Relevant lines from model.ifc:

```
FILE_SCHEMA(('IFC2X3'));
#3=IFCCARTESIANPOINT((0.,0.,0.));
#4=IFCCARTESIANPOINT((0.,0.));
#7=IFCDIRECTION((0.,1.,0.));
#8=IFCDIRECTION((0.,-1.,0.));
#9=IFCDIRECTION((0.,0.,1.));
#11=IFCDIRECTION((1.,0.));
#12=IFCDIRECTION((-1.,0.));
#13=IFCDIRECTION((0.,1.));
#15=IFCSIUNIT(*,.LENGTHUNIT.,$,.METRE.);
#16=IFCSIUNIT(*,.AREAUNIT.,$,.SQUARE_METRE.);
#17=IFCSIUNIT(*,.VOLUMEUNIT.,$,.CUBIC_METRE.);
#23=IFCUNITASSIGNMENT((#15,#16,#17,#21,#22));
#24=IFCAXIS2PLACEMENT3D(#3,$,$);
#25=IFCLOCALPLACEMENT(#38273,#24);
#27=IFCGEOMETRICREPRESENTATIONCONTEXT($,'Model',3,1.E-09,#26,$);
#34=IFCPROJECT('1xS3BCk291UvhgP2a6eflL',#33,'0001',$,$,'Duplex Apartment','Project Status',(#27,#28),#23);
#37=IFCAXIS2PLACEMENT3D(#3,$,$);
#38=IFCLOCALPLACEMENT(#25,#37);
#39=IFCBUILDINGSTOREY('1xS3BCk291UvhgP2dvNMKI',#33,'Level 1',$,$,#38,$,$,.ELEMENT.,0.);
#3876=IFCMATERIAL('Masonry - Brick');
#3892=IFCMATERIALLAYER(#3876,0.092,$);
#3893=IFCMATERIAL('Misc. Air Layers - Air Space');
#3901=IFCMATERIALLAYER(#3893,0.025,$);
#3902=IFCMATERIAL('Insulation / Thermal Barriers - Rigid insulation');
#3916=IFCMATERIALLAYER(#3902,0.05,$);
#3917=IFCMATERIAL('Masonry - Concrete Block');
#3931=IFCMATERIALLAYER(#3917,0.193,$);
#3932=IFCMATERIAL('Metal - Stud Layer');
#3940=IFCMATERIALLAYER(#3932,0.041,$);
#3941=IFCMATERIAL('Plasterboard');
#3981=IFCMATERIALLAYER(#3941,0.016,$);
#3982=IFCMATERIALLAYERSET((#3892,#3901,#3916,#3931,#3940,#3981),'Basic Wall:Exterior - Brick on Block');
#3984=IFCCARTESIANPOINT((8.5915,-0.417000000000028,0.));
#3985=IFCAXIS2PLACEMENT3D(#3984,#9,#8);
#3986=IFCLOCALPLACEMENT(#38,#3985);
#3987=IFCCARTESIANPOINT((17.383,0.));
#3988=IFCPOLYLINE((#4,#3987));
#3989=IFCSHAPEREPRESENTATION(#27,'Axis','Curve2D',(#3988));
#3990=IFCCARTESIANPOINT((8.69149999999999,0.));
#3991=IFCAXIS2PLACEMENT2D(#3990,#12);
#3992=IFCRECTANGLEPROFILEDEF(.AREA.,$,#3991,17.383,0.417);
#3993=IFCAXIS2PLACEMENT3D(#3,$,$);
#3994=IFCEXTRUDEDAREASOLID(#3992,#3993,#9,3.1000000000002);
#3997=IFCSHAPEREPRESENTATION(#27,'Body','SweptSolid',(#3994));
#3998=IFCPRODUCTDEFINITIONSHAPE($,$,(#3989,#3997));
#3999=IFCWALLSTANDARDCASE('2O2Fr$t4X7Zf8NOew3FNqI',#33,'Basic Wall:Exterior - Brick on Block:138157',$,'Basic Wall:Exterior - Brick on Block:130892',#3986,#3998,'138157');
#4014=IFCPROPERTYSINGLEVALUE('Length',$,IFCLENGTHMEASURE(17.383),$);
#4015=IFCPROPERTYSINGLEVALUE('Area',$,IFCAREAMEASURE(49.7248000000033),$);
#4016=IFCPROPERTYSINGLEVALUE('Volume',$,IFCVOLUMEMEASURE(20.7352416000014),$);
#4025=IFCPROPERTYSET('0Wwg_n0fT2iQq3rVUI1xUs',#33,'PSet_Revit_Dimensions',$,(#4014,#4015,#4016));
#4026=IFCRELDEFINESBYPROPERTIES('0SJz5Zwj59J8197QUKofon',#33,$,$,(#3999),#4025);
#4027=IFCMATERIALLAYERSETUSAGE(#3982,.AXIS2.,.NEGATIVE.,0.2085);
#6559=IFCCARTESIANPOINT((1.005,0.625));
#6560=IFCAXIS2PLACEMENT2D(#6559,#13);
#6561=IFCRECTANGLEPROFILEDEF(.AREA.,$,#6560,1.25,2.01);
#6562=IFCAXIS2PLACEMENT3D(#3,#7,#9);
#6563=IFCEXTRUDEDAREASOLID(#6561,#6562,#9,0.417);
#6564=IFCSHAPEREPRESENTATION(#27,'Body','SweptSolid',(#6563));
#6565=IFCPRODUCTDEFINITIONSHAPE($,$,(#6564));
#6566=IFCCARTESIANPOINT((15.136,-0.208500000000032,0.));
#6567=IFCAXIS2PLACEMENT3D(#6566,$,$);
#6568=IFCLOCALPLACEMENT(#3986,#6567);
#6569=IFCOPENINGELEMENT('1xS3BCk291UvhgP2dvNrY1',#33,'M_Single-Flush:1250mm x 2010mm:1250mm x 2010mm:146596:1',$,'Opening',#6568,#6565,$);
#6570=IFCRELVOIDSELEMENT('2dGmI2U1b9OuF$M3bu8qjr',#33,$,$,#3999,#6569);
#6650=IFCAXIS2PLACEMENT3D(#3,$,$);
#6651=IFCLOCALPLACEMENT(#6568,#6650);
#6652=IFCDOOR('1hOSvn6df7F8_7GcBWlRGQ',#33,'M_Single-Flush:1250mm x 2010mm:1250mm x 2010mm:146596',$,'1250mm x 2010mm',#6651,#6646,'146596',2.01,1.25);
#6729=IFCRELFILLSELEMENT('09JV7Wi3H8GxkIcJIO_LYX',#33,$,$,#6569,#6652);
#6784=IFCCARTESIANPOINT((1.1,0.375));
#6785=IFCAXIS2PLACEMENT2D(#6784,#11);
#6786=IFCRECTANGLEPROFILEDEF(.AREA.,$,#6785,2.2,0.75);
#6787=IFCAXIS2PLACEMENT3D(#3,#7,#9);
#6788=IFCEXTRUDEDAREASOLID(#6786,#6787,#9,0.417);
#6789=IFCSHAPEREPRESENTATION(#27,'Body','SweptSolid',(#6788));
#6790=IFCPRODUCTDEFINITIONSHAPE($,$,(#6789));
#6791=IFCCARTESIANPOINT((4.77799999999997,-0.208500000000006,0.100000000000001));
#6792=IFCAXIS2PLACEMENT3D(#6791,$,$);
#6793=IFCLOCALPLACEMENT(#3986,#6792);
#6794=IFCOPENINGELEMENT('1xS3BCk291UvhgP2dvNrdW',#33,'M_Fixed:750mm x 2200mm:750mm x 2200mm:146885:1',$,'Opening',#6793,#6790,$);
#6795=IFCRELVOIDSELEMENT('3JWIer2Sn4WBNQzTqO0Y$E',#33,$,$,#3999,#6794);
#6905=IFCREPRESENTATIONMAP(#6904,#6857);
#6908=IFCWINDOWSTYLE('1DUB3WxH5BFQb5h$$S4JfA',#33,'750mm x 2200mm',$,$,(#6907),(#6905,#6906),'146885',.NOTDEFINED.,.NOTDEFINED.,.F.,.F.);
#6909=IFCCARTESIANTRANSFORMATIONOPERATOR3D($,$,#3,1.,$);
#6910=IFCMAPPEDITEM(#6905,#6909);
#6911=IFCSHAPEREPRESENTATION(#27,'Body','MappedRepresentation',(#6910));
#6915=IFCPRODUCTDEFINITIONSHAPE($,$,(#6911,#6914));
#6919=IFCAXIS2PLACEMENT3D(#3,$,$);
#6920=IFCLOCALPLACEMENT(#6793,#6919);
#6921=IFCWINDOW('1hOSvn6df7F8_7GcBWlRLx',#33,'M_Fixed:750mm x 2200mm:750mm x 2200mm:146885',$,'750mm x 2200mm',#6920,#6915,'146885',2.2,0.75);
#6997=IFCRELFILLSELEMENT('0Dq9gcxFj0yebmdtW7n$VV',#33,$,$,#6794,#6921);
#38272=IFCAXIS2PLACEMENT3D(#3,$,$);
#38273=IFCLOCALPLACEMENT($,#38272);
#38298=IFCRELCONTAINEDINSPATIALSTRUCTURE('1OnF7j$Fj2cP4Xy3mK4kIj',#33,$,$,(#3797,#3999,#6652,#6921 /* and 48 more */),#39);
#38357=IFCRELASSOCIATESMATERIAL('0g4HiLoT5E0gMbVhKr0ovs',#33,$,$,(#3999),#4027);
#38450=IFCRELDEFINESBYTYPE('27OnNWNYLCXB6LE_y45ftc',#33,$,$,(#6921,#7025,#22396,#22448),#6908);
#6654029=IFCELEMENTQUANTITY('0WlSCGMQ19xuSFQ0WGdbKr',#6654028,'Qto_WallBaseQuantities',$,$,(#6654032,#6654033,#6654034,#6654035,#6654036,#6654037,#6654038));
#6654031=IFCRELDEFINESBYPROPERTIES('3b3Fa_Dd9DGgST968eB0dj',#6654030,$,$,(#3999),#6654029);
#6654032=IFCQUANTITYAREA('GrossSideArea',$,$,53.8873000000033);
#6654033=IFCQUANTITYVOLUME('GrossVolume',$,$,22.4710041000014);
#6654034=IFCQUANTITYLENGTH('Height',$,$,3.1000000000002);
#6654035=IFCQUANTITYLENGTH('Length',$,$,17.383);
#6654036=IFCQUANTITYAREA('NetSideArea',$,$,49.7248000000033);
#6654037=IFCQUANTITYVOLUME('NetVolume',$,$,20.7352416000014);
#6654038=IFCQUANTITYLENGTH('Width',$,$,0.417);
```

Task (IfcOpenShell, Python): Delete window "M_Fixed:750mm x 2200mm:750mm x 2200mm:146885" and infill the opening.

```python
import ifcopenshell
import ifcopenshell.api.feature
import ifcopenshell.api.pset
import ifcopenshell.api.root
import ifcopenshell.geom
import ifcopenshell.util.element
import ifcopenshell.util.shape
import ifcopenshell.util.unit

model = ifcopenshell.open("model.ifc")
area_scale = ifcopenshell.util.unit.calculate_unit_scale(model, "AREAUNIT")
volume_scale = ifcopenshell.util.unit.calculate_unit_scale(model, "VOLUMEUNIT")
settings = ifcopenshell.geom.settings()


def volume(element):
    """Net volume in cubic metres, openings subtracted."""
    shape = ifcopenshell.geom.create_shape(settings, element)
    return ifcopenshell.util.shape.get_volume(shape.geometry)


window = model.by_guid("1hOSvn6df7F8_7GcBWlRLx")
opening = window.FillsVoids[0].RelatingOpeningElement
wall = opening.VoidsElements[0].RelatingBuildingElement
before = volume(wall)

ifcopenshell.api.root.remove_product(model, product=window)
ifcopenshell.api.feature.remove_feature(model, feature=opening)

after = volume(wall)
thickness = 0.417  # wall thickness in metres

# Update the wall's stored quantities.
pset = model.by_id(ifcopenshell.util.element.get_pset(wall, "PSet_Revit_Dimensions", should_inherit=False)["id"])
ifcopenshell.api.pset.edit_pset(model, pset=pset, properties={
    "Area": model.create_entity("IfcAreaMeasure", after / thickness / area_scale),
    "Volume": model.create_entity("IfcVolumeMeasure", after / volume_scale),
})
qto = model.by_id(ifcopenshell.util.element.get_pset(wall, "Qto_WallBaseQuantities", should_inherit=False)["id"])
ifcopenshell.api.pset.edit_qto(model, qto=qto, properties={
    "NetSideArea": after / thickness / area_scale,
    "NetVolume": after / volume_scale,
})

print(f"wall volume {before:.3f} -> {after:.3f} m3")

model.write("model_updated.ifc")
```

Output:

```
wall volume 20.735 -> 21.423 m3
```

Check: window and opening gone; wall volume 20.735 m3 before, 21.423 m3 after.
